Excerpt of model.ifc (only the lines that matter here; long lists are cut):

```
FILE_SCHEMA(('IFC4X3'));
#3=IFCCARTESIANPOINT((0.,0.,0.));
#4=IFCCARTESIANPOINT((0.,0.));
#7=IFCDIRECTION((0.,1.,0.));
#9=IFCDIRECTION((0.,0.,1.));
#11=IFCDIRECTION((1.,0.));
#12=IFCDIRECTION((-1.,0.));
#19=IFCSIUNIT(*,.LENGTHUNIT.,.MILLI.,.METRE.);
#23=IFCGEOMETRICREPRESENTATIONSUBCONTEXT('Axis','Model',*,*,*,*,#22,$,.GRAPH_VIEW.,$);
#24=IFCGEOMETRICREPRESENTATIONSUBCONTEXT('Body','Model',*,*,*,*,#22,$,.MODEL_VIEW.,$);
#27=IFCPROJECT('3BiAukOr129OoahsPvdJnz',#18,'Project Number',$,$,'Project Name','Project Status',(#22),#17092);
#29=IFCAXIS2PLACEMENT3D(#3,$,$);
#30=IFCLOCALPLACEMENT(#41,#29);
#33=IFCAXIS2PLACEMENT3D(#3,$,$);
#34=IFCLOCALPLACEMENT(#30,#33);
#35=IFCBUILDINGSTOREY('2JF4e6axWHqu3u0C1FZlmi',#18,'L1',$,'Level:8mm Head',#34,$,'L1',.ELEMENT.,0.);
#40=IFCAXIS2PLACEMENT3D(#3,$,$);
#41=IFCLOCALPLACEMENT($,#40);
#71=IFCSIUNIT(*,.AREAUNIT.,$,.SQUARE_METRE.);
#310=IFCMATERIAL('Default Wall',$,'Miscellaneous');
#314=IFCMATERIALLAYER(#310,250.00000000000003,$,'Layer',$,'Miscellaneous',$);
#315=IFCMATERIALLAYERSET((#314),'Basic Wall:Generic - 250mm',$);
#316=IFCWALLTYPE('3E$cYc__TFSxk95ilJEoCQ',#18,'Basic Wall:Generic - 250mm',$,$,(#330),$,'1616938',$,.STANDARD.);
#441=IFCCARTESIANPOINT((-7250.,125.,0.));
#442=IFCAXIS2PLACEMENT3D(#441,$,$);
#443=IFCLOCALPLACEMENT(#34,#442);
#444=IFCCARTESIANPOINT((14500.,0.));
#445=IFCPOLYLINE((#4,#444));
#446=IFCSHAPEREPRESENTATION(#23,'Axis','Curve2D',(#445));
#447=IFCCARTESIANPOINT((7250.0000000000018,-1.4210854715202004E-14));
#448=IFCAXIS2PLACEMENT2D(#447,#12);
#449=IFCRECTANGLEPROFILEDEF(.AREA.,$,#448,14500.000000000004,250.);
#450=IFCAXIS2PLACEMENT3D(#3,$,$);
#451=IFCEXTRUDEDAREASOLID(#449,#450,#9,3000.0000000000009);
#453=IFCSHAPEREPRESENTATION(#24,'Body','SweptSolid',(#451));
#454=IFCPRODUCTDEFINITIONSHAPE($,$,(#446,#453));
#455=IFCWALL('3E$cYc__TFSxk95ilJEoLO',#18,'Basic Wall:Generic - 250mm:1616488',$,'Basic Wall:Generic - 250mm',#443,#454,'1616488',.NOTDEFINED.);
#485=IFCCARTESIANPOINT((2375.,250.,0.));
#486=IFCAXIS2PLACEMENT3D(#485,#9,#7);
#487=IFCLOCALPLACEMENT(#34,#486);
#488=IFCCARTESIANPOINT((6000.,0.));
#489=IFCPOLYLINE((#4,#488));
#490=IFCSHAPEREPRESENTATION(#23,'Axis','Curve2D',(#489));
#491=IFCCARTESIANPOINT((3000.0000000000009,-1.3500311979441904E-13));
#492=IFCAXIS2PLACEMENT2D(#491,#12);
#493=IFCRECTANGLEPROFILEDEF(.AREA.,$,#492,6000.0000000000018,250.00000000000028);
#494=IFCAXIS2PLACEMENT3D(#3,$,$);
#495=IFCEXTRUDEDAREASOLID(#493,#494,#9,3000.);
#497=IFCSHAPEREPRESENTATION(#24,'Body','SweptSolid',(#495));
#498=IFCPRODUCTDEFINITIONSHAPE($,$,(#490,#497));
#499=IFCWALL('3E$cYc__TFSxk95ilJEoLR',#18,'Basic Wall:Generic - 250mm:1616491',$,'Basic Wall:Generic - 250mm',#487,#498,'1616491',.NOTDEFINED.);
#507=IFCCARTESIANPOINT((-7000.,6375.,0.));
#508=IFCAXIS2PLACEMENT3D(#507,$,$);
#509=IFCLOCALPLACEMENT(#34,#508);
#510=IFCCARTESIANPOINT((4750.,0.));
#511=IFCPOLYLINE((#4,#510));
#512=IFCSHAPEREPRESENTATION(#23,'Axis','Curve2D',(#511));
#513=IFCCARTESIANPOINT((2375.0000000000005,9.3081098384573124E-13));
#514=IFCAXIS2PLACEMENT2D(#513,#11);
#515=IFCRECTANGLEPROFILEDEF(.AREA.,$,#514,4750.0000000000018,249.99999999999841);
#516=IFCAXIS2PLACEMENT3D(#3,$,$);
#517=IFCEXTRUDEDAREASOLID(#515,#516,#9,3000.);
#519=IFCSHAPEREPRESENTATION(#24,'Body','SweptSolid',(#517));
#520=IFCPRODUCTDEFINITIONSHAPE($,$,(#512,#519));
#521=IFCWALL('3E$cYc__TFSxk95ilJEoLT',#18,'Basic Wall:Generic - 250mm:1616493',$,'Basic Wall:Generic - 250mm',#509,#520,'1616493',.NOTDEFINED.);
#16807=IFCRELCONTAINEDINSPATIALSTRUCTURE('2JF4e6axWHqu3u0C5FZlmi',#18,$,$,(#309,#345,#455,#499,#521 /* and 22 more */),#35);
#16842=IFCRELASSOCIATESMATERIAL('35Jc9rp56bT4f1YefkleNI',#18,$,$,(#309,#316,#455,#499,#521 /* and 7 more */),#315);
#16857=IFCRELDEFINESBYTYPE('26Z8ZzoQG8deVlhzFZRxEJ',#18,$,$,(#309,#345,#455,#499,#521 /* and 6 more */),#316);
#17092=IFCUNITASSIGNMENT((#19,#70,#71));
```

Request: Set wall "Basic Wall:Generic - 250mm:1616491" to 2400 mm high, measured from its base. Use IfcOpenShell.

```python
import ifcopenshell
import ifcopenshell.geom
import ifcopenshell.util.representation
import ifcopenshell.util.shape
import ifcopenshell.util.unit

model = ifcopenshell.open("model.ifc")
unit_scale = ifcopenshell.util.unit.calculate_unit_scale(model)
settings = ifcopenshell.geom.settings()


def volume(element):
    """Net volume in cubic metres, openings subtracted."""
    shape = ifcopenshell.geom.create_shape(settings, element)
    return ifcopenshell.util.shape.get_volume(shape.geometry)


wall = model.by_id(499)
before = volume(wall)

body = ifcopenshell.util.representation.get_representation(wall, "Model", "Body")
solid = body.Items[0]
old_height = solid.Depth
solid.Depth = 2.4 / unit_scale
after = volume(wall)

print(f"height {old_height:g} -> {solid.Depth:g}, volume {before:.3f} -> {after:.3f} m3")

model.write("model-out.ifc")
```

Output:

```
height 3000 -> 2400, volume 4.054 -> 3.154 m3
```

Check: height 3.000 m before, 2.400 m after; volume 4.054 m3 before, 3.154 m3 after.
